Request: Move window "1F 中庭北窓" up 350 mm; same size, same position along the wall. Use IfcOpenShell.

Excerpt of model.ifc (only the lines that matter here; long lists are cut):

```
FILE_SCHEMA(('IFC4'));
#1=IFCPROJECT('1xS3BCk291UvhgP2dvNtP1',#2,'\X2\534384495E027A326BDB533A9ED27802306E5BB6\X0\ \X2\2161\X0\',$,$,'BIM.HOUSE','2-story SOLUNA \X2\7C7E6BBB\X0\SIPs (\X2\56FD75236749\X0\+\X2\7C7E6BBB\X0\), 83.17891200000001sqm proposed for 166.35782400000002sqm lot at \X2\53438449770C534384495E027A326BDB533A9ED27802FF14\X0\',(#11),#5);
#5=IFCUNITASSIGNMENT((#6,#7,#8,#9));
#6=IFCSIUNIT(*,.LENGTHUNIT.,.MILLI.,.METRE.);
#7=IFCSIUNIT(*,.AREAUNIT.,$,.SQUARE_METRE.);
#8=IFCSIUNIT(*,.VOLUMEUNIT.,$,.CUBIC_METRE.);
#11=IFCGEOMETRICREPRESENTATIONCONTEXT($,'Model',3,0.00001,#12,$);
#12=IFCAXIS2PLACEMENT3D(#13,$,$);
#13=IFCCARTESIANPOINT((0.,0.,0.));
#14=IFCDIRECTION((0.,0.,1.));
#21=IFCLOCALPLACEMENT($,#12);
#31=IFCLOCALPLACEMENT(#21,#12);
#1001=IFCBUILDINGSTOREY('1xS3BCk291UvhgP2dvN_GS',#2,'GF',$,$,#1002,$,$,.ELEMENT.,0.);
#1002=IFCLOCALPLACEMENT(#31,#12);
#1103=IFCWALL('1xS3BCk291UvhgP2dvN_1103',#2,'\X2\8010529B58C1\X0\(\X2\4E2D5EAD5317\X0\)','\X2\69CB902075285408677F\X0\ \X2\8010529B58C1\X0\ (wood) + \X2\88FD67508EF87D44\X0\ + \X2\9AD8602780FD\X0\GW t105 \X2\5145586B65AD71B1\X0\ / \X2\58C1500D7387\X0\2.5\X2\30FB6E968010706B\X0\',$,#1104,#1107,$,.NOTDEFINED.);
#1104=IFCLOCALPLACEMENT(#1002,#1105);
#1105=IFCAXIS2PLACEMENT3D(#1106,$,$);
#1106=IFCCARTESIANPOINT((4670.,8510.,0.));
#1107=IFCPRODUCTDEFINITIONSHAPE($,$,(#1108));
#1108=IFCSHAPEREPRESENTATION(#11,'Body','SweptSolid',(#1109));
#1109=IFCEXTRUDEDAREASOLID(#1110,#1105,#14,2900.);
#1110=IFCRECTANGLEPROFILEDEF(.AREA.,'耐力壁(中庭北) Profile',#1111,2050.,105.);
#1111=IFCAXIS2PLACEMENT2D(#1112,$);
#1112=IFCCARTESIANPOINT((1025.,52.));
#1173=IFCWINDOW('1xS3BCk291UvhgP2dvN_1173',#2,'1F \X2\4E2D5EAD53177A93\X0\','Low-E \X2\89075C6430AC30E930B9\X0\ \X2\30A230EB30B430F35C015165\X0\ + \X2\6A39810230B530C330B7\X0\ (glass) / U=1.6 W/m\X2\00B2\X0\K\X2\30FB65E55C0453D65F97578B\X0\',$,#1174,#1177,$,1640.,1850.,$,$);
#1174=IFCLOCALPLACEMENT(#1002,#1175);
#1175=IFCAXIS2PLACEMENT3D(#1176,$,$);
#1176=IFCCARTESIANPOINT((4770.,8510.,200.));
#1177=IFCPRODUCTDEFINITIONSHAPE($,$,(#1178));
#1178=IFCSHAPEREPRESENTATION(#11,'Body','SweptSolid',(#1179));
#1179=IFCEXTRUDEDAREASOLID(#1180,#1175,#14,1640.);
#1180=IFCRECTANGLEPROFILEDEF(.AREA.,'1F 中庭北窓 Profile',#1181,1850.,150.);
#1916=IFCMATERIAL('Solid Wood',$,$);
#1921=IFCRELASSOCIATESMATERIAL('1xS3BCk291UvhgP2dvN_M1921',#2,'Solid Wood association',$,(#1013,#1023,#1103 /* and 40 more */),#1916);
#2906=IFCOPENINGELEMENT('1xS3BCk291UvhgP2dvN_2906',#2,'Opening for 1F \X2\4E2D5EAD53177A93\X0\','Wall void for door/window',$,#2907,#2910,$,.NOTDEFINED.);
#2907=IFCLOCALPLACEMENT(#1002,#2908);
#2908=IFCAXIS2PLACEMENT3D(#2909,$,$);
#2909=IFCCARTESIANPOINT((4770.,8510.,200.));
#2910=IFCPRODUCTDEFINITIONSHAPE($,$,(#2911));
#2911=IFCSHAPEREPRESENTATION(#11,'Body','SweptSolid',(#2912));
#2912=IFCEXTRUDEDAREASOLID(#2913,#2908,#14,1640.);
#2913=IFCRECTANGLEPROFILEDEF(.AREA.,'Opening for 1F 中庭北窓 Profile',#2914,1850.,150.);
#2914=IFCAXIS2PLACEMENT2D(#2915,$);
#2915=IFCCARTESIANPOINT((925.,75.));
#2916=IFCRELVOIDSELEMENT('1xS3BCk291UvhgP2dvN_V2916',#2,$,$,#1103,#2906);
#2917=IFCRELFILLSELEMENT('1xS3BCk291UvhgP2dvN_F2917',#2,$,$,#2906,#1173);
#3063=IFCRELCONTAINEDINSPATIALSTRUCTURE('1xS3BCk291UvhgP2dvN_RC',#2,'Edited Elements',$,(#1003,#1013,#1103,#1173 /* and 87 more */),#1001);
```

```python
import numpy as np
import ifcopenshell
import ifcopenshell.api.geometry
import ifcopenshell.util.placement
import ifcopenshell.util.unit

model = ifcopenshell.open("model.ifc")
unit_scale = ifcopenshell.util.unit.calculate_unit_scale(model)

window = model.by_guid("1xS3BCk291UvhgP2dvN_1173")
opening = window.FillsVoids[0].RelatingOpeningElement
dz = 0.35 / unit_scale

shift = np.array([0.0, 0.0, dz])
# The window is not placed relative to its opening, so move both.
for product in (opening, window):
    matrix = ifcopenshell.util.placement.get_local_placement(product.ObjectPlacement)
    matrix[:3, 3] += shift
    ifcopenshell.api.geometry.edit_object_placement(model, product=product, matrix=matrix, is_si=False)

print(f"moved by {dz * unit_scale:+.3f} m")

model.write("model_updated.ifc")
```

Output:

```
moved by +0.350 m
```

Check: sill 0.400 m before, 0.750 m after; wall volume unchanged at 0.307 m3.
